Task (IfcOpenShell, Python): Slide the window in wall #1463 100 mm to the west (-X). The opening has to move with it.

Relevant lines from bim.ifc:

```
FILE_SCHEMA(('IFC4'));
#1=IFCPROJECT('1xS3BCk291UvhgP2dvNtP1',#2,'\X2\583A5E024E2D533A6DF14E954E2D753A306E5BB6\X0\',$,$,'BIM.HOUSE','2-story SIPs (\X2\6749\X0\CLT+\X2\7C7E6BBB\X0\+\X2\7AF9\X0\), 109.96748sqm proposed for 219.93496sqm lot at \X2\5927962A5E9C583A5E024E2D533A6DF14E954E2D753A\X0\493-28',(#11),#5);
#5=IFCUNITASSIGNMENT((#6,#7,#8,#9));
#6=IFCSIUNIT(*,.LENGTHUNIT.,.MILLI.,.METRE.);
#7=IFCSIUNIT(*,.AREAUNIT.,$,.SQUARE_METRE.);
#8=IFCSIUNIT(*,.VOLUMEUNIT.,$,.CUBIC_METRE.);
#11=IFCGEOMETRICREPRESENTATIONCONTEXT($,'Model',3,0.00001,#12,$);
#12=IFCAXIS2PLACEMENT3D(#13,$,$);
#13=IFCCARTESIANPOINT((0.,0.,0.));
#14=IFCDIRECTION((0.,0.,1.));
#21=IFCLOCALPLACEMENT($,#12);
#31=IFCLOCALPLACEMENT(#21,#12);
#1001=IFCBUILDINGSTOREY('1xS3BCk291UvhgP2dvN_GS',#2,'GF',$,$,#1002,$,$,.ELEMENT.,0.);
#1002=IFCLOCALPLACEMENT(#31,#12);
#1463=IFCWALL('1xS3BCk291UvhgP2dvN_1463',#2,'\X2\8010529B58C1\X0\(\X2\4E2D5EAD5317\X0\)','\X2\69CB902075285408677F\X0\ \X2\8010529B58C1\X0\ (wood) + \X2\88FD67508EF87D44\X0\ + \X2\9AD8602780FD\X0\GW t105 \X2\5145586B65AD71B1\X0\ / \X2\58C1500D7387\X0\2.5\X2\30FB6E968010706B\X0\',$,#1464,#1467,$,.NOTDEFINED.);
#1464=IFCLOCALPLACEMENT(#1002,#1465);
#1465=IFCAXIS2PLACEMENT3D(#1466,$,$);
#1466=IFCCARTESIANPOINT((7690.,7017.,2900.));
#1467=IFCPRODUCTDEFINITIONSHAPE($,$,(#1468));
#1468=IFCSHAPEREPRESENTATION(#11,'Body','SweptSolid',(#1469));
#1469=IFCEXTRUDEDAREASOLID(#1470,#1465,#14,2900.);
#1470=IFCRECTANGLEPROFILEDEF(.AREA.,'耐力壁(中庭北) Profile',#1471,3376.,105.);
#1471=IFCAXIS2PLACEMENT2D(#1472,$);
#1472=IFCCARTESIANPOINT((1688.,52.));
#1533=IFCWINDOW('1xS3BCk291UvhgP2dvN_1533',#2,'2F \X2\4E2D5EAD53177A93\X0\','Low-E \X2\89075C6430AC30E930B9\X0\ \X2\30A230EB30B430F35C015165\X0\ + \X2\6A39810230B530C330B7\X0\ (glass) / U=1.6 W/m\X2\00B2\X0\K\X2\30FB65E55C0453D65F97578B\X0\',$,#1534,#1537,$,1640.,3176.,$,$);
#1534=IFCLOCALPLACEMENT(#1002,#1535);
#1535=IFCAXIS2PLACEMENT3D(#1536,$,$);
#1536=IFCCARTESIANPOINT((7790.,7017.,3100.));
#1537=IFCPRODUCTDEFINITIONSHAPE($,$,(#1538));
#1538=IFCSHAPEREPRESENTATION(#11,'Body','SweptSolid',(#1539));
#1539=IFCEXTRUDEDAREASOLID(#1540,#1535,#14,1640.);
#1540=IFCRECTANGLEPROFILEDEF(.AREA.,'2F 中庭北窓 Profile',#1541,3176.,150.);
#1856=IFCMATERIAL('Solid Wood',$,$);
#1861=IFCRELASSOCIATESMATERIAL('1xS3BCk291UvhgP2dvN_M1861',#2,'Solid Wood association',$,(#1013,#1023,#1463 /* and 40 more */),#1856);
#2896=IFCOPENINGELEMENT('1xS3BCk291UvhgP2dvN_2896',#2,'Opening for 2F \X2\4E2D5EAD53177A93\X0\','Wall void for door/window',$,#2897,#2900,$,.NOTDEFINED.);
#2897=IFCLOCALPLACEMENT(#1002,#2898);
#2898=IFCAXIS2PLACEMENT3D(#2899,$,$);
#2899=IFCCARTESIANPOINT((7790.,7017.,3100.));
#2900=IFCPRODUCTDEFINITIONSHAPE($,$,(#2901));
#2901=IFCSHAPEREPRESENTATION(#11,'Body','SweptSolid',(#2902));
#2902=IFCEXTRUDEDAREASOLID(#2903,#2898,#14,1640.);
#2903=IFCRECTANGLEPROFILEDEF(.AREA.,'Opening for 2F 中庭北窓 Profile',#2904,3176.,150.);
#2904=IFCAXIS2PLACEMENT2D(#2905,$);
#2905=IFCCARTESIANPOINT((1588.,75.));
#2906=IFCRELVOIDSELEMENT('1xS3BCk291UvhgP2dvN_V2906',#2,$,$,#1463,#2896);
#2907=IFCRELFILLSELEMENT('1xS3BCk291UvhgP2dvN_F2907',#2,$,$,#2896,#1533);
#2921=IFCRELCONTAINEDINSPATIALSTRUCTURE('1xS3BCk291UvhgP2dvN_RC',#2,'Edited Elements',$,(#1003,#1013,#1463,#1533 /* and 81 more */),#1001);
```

```python
import ifcopenshell
import ifcopenshell.api.geometry
import ifcopenshell.util.placement
import ifcopenshell.util.unit

model = ifcopenshell.open("bim.ifc")
unit_scale = ifcopenshell.util.unit.calculate_unit_scale(model)

window = model.by_id(1533)
opening = window.FillsVoids[0].RelatingOpeningElement
wall = opening.VoidsElements[0].RelatingBuildingElement

wall_matrix = ifcopenshell.util.placement.get_local_placement(wall.ObjectPlacement)
shift = wall_matrix[:3, 0] * -0.1 / unit_scale
before = ifcopenshell.util.placement.get_local_placement(window.ObjectPlacement)[:3, 3].copy()

# The window is not placed relative to its opening, so move both.
for product in (opening, window):
    matrix = ifcopenshell.util.placement.get_local_placement(product.ObjectPlacement)
    matrix[:3, 3] += shift
    ifcopenshell.api.geometry.edit_object_placement(model, product=product, matrix=matrix, is_si=False)

after = ifcopenshell.util.placement.get_local_placement(window.ObjectPlacement)[:3, 3]
print("window moved by", (after - before).round(3) + 0.0)

model.write("bim_updated.ifc")
```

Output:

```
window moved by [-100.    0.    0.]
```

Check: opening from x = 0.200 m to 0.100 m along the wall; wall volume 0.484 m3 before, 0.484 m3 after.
